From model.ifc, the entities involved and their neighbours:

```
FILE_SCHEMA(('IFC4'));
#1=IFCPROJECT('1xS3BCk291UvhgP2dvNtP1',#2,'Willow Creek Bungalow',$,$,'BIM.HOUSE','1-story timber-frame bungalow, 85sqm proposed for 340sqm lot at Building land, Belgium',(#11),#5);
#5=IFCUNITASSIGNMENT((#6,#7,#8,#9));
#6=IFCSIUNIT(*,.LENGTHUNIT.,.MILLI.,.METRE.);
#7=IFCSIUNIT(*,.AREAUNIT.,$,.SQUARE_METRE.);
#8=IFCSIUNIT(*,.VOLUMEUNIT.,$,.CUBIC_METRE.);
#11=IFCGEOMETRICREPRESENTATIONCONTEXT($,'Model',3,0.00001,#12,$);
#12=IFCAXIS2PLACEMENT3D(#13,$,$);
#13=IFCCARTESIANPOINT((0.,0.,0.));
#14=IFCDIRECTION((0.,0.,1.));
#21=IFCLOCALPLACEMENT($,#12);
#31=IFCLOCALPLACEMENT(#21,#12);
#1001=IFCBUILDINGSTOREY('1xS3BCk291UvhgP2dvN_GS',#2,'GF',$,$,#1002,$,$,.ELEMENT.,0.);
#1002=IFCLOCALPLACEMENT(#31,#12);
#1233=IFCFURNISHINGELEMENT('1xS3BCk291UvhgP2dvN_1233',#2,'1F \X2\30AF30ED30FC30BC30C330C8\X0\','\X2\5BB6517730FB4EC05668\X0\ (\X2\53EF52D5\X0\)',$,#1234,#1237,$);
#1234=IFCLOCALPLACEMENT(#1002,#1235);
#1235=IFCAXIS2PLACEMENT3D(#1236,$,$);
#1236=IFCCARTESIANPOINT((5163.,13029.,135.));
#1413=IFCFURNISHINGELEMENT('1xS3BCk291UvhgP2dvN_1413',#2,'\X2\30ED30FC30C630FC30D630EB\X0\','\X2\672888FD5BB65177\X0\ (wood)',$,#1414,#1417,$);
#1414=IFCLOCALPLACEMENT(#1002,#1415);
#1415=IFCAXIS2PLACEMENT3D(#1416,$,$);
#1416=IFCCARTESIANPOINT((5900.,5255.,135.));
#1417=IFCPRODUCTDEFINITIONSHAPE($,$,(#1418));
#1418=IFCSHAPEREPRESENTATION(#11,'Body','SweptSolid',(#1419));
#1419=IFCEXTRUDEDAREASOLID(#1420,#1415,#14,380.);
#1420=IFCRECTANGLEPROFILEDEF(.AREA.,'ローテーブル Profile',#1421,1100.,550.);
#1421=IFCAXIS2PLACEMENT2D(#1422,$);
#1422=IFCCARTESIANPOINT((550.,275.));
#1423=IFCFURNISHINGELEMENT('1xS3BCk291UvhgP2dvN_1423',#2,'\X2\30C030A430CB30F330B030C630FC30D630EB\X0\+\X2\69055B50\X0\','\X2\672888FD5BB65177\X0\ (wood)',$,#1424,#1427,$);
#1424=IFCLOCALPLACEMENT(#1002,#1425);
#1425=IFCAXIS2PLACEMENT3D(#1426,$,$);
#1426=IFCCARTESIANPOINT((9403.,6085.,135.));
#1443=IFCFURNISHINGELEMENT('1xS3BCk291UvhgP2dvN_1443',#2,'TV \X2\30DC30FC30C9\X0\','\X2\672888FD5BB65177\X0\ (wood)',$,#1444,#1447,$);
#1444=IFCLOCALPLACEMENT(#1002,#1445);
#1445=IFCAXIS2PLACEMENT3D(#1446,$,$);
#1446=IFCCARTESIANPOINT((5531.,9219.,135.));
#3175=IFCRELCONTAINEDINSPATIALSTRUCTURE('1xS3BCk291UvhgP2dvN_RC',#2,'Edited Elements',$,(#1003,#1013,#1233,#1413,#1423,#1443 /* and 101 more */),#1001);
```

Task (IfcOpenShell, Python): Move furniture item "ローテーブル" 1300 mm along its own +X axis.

```python
import ifcopenshell
import ifcopenshell.api.geometry
import ifcopenshell.util.placement
import ifcopenshell.util.unit

model = ifcopenshell.open("model.ifc")
unit_scale = ifcopenshell.util.unit.calculate_unit_scale(model)

item = model.by_guid("1xS3BCk291UvhgP2dvN_1413")
matrix = ifcopenshell.util.placement.get_local_placement(item.ObjectPlacement)
matrix[:3, 3] += matrix[:3, 0] * 1.3 / unit_scale
ifcopenshell.api.geometry.edit_object_placement(model, product=item, matrix=matrix, is_si=False)

print(ifcopenshell.util.placement.get_local_placement(item.ObjectPlacement).round(3) + 0.0)

model.write("model_edited.ifc")
```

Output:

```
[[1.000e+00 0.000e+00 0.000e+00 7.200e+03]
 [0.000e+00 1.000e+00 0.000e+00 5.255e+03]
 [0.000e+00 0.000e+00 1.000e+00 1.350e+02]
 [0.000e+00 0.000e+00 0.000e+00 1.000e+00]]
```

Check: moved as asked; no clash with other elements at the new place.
